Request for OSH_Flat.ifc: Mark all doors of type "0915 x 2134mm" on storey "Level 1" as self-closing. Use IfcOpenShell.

First a look at what the model holds.

```python
import ifcopenshell
import ifcopenshell.util.element

model = ifcopenshell.open("OSH_Flat.ifc")
print(model.schema)
storey = next(s for s in model.by_type("IfcBuildingStorey") if s.Name == "Level 1")
doors = [e for e in ifcopenshell.util.element.get_decomposition(storey) if e.is_a("IfcDoor")]
seen = {}
for e in doors:
    element_type = ifcopenshell.util.element.get_type(e)
    key = (element_type.Name if element_type != e and element_type else None, ifcopenshell.util.element.get_pset(e, "Pset_DoorCommon", "SelfClosing"))
    seen[key] = seen.get(key, 0) + 1
for (name, value), count in sorted(seen.items(), key=str):
    print(count, "x", name, "|", value)
```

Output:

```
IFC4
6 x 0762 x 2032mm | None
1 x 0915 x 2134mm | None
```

```python
import ifcopenshell
import ifcopenshell.api.pset
import ifcopenshell.util.element

model = ifcopenshell.open("OSH_Flat.ifc")

storey = next(s for s in model.by_type("IfcBuildingStorey") if s.Name == "Level 1")
doors = [e for e in ifcopenshell.util.element.get_decomposition(storey) if e.is_a("IfcDoor")]

count = 0
for e in doors:
    element_type = ifcopenshell.util.element.get_type(e)
    if element_type in (None, e) or element_type.Name != "0915 x 2134mm":
        continue
    # add_pset returns the element's existing set when there is one.
    pset = ifcopenshell.api.pset.add_pset(model, product=e, name="Pset_DoorCommon")
    ifcopenshell.api.pset.edit_pset(model, pset=pset, properties={"SelfClosing": True})
    count += 1

print(count, "doors updated")

model.write("OSH_Flat-out.ifc")
```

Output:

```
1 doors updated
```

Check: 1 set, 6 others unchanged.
